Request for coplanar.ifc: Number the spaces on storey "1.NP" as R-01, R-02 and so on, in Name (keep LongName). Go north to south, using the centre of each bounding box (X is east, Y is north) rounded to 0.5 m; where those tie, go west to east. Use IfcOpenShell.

First a look at what the model holds.

```python
import ifcopenshell
import ifcopenshell.util.element
import ifcopenshell.util.placement

model = ifcopenshell.open("coplanar.ifc")
print(model.schema)
storey = next(s for s in model.by_type("IfcBuildingStorey") if s.Name == "1.NP")
spaces = [e for e in ifcopenshell.util.element.get_decomposition(storey) if e.is_a("IfcSpace")]
for e in sorted(spaces, key=lambda e: e.id()):
    origin = ifcopenshell.util.placement.get_local_placement(e.ObjectPlacement)[:3, 3]
    print(e.id(), e.Name, e.LongName, origin.round(2) + 0.0, sep=" | ")
```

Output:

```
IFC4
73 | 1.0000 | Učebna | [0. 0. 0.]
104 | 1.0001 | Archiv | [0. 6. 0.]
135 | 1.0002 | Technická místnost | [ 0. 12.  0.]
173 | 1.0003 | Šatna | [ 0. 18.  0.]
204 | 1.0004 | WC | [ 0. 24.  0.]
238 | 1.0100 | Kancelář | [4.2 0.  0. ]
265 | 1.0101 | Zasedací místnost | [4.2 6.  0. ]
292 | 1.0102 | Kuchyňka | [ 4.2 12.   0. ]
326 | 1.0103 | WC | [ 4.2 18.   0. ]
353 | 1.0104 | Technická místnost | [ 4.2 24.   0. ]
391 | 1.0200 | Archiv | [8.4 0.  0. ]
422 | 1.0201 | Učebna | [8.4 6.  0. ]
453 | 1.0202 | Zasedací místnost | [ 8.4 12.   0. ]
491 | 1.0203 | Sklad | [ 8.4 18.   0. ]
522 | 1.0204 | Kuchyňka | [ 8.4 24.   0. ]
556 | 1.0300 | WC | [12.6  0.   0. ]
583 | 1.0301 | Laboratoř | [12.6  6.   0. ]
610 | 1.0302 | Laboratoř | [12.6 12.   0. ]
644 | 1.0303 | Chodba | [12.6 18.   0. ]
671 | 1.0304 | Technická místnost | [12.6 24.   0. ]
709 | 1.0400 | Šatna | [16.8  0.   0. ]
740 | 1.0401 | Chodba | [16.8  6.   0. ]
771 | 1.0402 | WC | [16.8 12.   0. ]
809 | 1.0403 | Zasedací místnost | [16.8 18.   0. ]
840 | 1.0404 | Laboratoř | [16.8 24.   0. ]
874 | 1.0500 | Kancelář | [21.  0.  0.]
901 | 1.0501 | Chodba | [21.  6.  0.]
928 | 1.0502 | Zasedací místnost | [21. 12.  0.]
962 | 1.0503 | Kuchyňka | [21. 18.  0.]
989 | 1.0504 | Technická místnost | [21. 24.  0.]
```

```python
import ifcopenshell
import ifcopenshell.geom
import ifcopenshell.util.element
import ifcopenshell.util.shape

model = ifcopenshell.open("coplanar.ifc")
settings = ifcopenshell.geom.settings()
settings.set("use-world-coords", True)


def centre(element):
    shape = ifcopenshell.geom.create_shape(settings, element)
    return ifcopenshell.util.shape.get_bbox_centroid(shape.geometry)


storey = next(s for s in model.by_type("IfcBuildingStorey") if s.Name == "1.NP")
spaces = [e for e in ifcopenshell.util.element.get_decomposition(storey) if e.is_a("IfcSpace")]

# Insertion points can sit at a corner or the storey origin, so sort by the geometry (in metres).
centres = {e: centre(e) for e in spaces}
spaces.sort(key=lambda e: (-round(centres[e][1] / 0.5), centres[e][0]))

for i, e in enumerate(spaces, start=1):
    number = f"R-{i:02d}"
    e.Name = number
    print(e.id(), number)

model.write("coplanar_rev.ifc")
```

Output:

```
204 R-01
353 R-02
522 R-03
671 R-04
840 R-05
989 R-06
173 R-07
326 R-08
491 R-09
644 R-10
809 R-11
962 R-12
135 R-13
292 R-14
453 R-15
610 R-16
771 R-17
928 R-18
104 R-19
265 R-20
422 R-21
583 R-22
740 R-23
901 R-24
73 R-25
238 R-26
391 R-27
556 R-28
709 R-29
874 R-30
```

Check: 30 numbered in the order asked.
